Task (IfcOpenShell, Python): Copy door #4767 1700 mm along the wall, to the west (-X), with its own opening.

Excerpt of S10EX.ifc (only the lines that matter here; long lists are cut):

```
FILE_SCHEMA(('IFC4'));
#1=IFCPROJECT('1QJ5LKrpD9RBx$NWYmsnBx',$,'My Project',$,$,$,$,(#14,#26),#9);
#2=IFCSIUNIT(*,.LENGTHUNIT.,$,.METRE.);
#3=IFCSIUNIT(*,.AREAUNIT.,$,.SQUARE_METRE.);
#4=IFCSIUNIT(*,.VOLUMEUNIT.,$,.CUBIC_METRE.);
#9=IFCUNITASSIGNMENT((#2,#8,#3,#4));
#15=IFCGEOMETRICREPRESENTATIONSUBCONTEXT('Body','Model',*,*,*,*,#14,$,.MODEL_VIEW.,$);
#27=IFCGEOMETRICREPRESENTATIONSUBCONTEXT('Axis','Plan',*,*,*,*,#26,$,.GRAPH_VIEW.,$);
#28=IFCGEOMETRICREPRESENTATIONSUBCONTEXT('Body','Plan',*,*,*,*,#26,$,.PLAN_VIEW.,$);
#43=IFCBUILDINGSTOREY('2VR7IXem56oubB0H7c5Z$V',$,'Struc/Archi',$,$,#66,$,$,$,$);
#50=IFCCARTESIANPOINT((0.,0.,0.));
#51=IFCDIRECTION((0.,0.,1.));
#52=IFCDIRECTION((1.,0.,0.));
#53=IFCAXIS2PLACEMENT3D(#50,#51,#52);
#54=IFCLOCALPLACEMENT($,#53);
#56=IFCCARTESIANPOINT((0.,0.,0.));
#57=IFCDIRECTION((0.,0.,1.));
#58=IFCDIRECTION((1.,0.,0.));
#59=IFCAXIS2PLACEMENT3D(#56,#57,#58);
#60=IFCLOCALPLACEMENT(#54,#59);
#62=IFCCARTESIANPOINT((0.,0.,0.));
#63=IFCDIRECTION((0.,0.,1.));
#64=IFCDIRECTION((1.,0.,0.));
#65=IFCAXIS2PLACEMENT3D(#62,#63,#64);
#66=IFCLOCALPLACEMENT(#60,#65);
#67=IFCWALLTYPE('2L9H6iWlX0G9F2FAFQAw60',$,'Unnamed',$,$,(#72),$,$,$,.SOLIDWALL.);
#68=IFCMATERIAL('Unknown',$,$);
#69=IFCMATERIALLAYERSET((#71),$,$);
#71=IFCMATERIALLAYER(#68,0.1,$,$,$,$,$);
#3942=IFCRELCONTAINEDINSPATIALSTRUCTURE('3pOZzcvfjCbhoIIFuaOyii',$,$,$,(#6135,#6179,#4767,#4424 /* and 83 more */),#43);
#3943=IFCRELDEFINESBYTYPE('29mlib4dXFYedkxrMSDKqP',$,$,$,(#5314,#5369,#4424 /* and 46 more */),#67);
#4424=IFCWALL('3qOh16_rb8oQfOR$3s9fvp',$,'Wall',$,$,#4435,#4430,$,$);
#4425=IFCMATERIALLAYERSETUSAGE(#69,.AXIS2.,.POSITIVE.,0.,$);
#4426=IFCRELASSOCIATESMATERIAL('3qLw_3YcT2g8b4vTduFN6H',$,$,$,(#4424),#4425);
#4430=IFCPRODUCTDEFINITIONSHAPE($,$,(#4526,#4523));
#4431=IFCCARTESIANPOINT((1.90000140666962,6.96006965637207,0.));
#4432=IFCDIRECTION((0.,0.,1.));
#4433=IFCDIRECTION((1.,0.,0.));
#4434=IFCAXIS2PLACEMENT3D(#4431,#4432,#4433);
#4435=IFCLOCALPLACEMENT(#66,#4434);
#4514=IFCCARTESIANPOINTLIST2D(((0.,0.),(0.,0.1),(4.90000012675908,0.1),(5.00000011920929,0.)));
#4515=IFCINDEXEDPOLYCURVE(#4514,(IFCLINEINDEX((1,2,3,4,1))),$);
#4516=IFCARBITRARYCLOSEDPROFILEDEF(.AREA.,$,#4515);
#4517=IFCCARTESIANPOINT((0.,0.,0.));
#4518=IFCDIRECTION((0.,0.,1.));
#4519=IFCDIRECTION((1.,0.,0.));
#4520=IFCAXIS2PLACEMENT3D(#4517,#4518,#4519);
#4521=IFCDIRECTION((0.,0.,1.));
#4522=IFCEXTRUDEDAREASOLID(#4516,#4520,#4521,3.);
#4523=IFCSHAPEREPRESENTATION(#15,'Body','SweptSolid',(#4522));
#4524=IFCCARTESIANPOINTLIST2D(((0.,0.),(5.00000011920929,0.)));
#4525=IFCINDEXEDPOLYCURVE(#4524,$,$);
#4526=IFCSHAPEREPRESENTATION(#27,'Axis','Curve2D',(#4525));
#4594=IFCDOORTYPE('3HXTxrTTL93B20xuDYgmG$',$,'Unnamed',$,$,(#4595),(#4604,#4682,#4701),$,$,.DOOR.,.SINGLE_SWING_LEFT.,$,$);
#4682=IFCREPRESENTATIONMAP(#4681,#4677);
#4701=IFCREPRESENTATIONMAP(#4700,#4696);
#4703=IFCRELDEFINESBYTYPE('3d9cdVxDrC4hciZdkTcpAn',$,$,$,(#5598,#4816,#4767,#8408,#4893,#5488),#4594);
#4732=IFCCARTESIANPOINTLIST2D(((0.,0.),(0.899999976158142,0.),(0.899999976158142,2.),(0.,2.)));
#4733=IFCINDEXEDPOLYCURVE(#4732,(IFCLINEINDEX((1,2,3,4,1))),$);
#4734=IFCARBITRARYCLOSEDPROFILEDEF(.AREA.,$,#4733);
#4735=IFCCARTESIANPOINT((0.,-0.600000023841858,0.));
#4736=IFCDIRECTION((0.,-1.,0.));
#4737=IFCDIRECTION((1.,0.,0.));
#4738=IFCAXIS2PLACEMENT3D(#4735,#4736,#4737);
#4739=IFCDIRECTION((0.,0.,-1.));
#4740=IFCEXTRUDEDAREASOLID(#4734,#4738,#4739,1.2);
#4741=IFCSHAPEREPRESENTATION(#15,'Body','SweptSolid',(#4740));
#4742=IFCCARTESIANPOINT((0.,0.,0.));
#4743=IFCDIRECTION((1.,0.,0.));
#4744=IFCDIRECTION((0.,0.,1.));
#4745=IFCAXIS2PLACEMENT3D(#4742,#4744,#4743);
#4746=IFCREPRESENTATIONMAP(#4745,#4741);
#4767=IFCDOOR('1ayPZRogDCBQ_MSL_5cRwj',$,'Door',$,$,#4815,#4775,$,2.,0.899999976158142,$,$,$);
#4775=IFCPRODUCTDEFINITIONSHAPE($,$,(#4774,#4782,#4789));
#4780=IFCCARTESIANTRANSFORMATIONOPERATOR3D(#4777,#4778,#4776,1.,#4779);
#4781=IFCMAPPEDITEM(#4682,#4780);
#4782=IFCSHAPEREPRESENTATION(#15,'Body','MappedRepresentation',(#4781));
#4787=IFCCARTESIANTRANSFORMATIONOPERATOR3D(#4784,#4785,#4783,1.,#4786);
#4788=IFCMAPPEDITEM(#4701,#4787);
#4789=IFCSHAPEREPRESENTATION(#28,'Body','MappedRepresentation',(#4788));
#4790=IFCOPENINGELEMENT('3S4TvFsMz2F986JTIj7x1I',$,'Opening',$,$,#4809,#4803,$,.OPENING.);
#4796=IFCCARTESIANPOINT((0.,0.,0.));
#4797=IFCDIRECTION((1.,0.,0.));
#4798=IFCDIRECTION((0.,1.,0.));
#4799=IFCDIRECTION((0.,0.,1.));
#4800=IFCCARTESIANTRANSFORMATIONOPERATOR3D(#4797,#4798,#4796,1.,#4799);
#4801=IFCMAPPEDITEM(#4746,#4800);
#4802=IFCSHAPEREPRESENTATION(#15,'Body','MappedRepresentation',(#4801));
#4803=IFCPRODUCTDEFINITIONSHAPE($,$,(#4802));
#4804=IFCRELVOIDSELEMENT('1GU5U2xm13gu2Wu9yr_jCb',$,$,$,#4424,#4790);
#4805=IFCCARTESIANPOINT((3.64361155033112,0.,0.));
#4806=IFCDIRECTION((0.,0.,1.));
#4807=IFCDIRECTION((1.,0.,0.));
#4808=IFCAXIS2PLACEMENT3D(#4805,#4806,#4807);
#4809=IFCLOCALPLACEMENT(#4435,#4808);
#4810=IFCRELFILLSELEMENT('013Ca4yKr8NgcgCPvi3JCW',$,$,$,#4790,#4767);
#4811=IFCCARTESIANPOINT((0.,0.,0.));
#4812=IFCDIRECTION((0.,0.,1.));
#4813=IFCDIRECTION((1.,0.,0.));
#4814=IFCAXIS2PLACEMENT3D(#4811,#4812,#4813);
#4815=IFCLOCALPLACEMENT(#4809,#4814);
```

```python
import ifcopenshell
import ifcopenshell.api.feature
import ifcopenshell.api.geometry
import ifcopenshell.api.root
import ifcopenshell.geom
import ifcopenshell.util.element
import ifcopenshell.util.placement
import ifcopenshell.util.shape

model = ifcopenshell.open("S10EX.ifc")
settings = ifcopenshell.geom.settings()


def volume(element):
    """Net volume in cubic metres, openings subtracted."""
    shape = ifcopenshell.geom.create_shape(settings, element)
    return ifcopenshell.util.shape.get_volume(shape.geometry)


door = model.by_guid("1ayPZRogDCBQ_MSL_5cRwj")
opening = door.FillsVoids[0].RelatingOpeningElement
wall = opening.VoidsElements[0].RelatingBuildingElement
before = volume(wall)
shift = ifcopenshell.util.placement.get_local_placement(wall.ObjectPlacement)[:3, 0] * -1.7

# copy_class copies the void relationship, type, container and properties, but no geometry.
new_opening = ifcopenshell.api.root.copy_class(model, product=opening)
new_opening.Representation = ifcopenshell.util.element.copy_deep(
    model, opening.Representation, exclude=["IfcGeometricRepresentationContext", "IfcRepresentationMap"]
)
new_door = ifcopenshell.api.root.copy_class(model, product=door)
new_door.Representation = ifcopenshell.util.element.copy_deep(
    model, door.Representation, exclude=["IfcGeometricRepresentationContext", "IfcRepresentationMap"]
)
ifcopenshell.api.feature.add_filling(model, opening=new_opening, element=new_door)

for old, new in ((opening, new_opening), (door, new_door)):
    matrix = ifcopenshell.util.placement.get_local_placement(old.ObjectPlacement)
    matrix[:3, 3] += shift
    ifcopenshell.api.geometry.edit_object_placement(model, product=new, matrix=matrix, is_si=False)

after = volume(wall)

print(f"wall volume {before:.3f} -> {after:.3f} m3")

model.write("S10EX-out.ifc")
```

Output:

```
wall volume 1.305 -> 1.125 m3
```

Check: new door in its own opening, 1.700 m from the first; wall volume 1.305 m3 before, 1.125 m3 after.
